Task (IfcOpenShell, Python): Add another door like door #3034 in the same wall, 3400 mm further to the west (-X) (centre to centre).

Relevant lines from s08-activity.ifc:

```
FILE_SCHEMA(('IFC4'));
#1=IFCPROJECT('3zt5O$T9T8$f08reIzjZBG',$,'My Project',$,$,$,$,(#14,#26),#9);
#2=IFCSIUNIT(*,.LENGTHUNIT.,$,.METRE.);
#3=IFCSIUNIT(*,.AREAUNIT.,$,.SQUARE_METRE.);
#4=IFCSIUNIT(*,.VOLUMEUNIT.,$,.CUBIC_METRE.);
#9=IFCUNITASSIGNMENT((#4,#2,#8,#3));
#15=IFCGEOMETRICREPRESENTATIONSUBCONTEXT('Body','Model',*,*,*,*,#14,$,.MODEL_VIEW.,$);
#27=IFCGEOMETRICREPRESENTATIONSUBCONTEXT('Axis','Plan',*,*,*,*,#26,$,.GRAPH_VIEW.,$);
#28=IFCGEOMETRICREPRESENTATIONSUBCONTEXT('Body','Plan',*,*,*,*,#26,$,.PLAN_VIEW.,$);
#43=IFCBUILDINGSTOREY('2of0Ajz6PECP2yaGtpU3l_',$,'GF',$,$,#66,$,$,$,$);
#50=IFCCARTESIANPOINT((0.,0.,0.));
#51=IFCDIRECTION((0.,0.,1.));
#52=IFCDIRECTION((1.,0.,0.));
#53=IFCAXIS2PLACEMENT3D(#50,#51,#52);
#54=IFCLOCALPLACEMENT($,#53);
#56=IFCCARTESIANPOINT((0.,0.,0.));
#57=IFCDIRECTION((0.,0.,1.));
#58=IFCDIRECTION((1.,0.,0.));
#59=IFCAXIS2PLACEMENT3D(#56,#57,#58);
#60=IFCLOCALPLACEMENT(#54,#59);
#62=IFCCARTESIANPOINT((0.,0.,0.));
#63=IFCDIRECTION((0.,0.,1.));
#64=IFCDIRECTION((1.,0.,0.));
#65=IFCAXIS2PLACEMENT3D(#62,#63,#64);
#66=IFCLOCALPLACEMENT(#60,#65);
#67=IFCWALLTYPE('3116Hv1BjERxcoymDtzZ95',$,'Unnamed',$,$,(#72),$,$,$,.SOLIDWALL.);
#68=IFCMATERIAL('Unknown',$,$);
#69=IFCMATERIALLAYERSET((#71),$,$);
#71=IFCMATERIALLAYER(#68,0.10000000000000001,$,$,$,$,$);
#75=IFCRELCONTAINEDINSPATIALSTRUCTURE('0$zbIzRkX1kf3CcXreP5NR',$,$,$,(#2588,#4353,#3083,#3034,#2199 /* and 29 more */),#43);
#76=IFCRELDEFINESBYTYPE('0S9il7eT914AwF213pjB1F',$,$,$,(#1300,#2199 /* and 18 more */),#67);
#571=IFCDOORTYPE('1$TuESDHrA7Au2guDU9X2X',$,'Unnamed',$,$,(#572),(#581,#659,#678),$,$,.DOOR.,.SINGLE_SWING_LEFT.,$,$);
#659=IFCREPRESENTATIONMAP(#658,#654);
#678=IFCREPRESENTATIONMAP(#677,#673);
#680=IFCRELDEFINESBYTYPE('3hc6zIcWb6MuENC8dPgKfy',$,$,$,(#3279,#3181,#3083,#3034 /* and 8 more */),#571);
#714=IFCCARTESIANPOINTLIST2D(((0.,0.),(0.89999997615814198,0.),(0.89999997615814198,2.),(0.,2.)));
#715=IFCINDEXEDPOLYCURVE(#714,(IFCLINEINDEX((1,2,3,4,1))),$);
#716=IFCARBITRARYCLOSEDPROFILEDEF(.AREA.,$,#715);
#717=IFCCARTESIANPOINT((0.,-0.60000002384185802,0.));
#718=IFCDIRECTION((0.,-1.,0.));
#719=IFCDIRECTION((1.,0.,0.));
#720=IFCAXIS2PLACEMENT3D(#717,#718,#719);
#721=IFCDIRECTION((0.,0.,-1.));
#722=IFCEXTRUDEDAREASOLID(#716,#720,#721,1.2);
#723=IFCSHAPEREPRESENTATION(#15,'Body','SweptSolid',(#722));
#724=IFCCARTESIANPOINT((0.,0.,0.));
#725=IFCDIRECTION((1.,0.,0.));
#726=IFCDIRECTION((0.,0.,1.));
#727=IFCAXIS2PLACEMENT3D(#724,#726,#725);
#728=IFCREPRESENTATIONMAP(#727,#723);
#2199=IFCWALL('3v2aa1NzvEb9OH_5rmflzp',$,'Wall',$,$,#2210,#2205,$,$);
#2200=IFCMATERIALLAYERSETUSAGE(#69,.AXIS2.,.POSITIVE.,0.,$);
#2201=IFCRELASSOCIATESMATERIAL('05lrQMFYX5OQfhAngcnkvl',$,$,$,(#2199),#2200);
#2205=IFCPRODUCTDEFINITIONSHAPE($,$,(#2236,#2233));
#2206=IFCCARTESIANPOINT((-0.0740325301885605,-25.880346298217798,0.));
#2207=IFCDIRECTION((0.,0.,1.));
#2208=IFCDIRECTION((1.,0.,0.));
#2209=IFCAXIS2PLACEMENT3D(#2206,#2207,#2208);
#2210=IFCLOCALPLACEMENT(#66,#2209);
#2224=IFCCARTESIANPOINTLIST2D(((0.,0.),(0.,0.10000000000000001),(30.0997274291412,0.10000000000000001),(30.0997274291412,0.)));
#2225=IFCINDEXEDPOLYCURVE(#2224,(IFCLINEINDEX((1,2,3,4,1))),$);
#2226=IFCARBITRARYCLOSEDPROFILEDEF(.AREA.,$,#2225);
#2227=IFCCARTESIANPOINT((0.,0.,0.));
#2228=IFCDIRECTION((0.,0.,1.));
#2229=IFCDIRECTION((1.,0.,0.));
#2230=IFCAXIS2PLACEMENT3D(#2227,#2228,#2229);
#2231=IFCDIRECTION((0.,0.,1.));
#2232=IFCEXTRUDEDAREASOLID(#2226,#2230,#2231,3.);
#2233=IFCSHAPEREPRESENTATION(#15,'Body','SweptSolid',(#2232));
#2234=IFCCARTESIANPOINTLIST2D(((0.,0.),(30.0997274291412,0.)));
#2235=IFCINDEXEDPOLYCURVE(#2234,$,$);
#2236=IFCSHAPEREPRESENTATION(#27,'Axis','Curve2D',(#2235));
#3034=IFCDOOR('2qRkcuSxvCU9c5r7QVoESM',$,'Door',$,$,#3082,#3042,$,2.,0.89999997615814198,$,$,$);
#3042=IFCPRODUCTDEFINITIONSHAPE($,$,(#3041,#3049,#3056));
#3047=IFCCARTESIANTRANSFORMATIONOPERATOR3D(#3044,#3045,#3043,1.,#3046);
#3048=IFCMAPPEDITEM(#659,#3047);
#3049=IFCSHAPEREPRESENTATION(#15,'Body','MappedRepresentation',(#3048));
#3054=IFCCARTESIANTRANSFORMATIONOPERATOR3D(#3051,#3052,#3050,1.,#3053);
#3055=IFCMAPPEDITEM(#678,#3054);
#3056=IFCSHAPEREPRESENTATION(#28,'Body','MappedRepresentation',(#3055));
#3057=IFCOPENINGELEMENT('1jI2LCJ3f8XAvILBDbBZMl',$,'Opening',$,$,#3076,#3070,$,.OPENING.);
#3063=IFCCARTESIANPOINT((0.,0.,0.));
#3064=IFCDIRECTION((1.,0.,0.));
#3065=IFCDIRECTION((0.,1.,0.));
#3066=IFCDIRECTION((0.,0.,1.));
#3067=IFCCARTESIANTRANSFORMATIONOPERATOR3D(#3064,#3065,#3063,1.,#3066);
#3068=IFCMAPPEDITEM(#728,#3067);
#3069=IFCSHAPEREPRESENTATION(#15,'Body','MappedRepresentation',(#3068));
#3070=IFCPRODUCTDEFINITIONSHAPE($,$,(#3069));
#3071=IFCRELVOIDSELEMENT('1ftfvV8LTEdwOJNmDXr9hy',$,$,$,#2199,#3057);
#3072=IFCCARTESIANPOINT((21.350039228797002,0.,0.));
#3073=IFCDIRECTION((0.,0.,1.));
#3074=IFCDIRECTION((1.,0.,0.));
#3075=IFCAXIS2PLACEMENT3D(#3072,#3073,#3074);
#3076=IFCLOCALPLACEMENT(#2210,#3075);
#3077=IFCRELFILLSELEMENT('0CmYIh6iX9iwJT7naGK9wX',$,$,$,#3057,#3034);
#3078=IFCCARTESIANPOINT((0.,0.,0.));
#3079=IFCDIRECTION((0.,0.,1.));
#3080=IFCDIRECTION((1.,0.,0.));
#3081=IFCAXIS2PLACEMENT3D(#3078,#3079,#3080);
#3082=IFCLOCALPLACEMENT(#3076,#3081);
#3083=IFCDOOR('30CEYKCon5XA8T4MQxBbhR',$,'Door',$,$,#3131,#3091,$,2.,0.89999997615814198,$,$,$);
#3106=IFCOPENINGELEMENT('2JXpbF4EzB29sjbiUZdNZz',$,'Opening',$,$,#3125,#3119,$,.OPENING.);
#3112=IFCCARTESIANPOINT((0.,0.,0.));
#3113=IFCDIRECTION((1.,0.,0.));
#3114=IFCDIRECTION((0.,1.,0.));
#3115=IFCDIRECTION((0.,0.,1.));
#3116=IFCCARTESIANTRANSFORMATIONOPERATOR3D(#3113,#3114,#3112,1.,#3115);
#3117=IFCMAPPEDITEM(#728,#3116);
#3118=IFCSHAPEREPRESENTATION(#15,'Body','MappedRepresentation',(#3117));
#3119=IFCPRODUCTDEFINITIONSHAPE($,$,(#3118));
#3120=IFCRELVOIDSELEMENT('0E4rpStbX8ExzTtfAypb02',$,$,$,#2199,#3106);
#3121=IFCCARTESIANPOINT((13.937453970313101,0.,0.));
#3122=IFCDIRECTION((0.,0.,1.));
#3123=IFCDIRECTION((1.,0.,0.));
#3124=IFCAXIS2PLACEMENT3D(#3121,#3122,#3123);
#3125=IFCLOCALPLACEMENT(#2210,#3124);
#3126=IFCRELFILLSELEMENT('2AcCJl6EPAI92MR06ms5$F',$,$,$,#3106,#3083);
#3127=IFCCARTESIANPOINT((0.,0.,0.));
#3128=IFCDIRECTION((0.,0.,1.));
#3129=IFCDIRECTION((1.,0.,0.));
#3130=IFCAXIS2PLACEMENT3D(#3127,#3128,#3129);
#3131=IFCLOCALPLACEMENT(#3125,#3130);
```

```python
import ifcopenshell
import ifcopenshell.api.feature
import ifcopenshell.api.geometry
import ifcopenshell.api.root
import ifcopenshell.geom
import ifcopenshell.util.element
import ifcopenshell.util.placement
import ifcopenshell.util.shape
import ifcopenshell.util.unit

model = ifcopenshell.open("s08-activity.ifc")
unit_scale = ifcopenshell.util.unit.calculate_unit_scale(model)
settings = ifcopenshell.geom.settings()


def volume(element):
    """Net volume in cubic metres, openings subtracted."""
    shape = ifcopenshell.geom.create_shape(settings, element)
    return ifcopenshell.util.shape.get_volume(shape.geometry)


door = model.by_id(3034)
opening = door.FillsVoids[0].RelatingOpeningElement
wall = opening.VoidsElements[0].RelatingBuildingElement
before = volume(wall)
shift = ifcopenshell.util.placement.get_local_placement(wall.ObjectPlacement)[:3, 0] * -3.4 / unit_scale

# copy_class copies the void relationship, type, container and properties, but no geometry.
new_opening = ifcopenshell.api.root.copy_class(model, product=opening)
new_opening.Representation = ifcopenshell.util.element.copy_deep(
    model, opening.Representation, exclude=["IfcGeometricRepresentationContext", "IfcRepresentationMap"]
)
new_door = ifcopenshell.api.root.copy_class(model, product=door)
new_door.Representation = ifcopenshell.util.element.copy_deep(
    model, door.Representation, exclude=["IfcGeometricRepresentationContext", "IfcRepresentationMap"]
)
ifcopenshell.api.feature.add_filling(model, opening=new_opening, element=new_door)

for old, new in ((opening, new_opening), (door, new_door)):
    matrix = ifcopenshell.util.placement.get_local_placement(old.ObjectPlacement)
    matrix[:3, 3] += shift
    ifcopenshell.api.geometry.edit_object_placement(model, product=new, matrix=matrix, is_si=False)

after = volume(wall)

print(f"wall volume {before:.3f} -> {after:.3f} m3")

model.write("s08-activity-out.ifc")
```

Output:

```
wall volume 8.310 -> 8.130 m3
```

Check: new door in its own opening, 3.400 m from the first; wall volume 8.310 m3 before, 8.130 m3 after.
